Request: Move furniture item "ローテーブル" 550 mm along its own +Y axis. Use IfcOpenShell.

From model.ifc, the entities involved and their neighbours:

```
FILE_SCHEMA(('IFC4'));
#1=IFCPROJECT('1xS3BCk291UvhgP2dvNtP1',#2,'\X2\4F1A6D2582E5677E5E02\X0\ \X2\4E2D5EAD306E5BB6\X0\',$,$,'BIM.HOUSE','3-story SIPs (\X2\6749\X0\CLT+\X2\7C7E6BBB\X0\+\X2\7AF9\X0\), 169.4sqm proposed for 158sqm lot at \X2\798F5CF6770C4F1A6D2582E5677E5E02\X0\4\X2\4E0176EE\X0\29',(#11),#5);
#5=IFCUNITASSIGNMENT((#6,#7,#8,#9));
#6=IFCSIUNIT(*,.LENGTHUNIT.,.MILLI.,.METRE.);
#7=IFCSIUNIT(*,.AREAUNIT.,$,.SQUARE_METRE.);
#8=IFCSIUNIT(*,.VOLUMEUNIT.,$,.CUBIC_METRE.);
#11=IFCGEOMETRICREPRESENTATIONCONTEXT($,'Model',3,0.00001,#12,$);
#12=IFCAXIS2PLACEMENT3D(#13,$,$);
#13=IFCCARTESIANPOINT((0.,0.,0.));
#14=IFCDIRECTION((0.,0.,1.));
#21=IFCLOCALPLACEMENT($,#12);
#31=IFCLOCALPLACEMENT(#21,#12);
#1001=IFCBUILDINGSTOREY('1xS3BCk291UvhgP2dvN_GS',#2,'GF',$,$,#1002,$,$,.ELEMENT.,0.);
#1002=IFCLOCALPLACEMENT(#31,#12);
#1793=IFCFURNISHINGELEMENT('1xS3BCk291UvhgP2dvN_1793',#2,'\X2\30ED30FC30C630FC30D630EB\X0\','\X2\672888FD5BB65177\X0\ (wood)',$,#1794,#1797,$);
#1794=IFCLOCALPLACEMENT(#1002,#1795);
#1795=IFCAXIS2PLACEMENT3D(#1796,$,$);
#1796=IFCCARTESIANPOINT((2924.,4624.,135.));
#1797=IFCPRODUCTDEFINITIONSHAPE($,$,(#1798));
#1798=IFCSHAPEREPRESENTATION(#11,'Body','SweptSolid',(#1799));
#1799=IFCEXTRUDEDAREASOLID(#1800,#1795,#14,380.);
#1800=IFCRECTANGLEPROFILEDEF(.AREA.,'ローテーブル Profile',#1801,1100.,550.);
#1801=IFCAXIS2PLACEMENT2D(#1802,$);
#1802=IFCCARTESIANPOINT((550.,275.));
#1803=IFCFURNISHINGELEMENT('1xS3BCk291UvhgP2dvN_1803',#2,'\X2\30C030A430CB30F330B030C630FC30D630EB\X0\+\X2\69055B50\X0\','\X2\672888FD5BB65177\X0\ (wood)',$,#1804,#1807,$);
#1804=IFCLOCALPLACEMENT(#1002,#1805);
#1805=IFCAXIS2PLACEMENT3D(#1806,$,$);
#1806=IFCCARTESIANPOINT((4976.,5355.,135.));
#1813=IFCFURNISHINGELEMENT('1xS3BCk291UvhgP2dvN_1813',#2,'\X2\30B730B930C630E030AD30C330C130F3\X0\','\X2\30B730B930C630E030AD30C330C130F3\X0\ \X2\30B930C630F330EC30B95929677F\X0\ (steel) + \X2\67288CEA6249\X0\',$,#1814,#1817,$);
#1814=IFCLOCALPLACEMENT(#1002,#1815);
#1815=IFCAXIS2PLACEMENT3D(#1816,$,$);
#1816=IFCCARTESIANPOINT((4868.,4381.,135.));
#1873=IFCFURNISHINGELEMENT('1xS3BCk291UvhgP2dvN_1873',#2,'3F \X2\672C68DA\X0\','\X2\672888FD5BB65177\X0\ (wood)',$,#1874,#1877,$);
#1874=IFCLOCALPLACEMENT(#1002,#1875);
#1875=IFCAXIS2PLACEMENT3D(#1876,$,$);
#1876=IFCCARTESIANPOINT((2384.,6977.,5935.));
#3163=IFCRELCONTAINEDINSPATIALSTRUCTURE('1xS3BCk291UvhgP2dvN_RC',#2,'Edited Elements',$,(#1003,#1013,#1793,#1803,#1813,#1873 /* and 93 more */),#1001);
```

```python
import ifcopenshell
import ifcopenshell.api.geometry
import ifcopenshell.util.placement

model = ifcopenshell.open("model.ifc")

item = model.by_guid("1xS3BCk291UvhgP2dvN_1793")
matrix = ifcopenshell.util.placement.get_local_placement(item.ObjectPlacement)
matrix[:3, 3] += matrix[:3, 1] * 550.0
ifcopenshell.api.geometry.edit_object_placement(model, product=item, matrix=matrix, is_si=False)

print(ifcopenshell.util.placement.get_local_placement(item.ObjectPlacement).round(3) + 0.0)

model.write("model_edited.ifc")
```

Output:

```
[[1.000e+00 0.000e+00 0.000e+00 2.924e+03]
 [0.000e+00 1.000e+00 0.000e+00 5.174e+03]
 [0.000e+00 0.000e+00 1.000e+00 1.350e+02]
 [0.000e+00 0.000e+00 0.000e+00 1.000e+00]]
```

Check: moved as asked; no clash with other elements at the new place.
